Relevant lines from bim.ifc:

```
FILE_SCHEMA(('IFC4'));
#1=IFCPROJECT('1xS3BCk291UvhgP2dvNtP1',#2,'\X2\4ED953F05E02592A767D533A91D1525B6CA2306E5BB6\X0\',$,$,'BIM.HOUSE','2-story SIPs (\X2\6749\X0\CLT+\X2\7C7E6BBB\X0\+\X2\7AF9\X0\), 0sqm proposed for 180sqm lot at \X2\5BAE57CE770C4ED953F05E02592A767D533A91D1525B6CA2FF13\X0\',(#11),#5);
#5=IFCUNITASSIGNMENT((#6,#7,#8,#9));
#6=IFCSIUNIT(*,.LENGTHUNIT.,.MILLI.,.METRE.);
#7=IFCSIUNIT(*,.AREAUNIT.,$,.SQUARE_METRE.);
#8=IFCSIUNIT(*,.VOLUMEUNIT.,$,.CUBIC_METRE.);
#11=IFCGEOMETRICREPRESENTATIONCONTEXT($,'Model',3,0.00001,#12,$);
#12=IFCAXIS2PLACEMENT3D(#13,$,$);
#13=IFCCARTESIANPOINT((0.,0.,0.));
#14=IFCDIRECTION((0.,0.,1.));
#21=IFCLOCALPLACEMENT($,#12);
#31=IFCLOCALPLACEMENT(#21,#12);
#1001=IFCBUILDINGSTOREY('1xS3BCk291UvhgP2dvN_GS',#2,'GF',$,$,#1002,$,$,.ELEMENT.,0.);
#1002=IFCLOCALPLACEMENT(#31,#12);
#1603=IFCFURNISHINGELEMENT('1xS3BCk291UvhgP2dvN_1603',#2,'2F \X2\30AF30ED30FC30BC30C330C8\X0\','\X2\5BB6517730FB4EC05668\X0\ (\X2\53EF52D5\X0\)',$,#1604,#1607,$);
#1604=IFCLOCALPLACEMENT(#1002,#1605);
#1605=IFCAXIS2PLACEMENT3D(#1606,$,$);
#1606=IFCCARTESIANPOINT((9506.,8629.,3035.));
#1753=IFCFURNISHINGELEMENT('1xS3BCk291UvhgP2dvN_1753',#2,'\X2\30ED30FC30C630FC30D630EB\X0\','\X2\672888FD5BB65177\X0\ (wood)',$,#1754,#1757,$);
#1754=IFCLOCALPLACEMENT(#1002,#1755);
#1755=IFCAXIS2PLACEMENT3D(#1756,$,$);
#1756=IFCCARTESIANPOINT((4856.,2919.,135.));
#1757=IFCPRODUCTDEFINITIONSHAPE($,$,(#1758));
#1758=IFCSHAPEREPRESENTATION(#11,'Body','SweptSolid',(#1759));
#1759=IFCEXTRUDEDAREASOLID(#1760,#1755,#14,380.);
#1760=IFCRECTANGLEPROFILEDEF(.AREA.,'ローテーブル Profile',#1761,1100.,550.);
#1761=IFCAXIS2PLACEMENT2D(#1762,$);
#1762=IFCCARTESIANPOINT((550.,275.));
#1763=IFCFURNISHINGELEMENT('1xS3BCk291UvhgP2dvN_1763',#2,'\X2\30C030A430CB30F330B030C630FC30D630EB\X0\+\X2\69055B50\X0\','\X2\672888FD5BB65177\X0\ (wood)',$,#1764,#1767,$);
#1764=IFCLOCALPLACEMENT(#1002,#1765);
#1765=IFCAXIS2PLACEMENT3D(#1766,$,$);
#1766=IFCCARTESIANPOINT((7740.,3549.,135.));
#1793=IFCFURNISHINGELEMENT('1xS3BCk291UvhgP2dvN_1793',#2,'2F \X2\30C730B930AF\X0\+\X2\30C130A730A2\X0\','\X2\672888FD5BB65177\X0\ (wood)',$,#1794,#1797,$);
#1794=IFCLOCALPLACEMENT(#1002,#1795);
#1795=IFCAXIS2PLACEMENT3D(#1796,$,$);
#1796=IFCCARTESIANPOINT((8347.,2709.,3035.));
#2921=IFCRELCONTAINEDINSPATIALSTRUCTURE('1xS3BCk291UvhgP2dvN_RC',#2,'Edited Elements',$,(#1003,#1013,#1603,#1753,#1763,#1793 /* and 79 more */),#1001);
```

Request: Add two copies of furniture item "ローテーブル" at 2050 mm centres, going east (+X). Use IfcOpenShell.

```python
import numpy as np
import ifcopenshell
import ifcopenshell.api.geometry
import ifcopenshell.api.root
import ifcopenshell.util.element
import ifcopenshell.util.placement
import ifcopenshell.util.unit

model = ifcopenshell.open("bim.ifc")
unit_scale = ifcopenshell.util.unit.calculate_unit_scale(model)


def reuse_history(source, copy):
    """copy_class also copies each property set's owner history, people and application; keep the originals."""
    for rel in copy.IsDefinedBy:
        if rel.is_a("IfcRelDefinesByProperties") and (history := rel.RelatingPropertyDefinition.OwnerHistory):
            rel.RelatingPropertyDefinition.OwnerHistory = source.OwnerHistory
            ifcopenshell.util.element.remove_deep2(model, history)


source = model.by_id(1753)
base = ifcopenshell.util.placement.get_local_placement(source.ObjectPlacement)
step = np.array([1.0, 0.0, 0.0]) * 2.05 / unit_scale

for i in range(1, 3):
    copy = ifcopenshell.api.root.copy_class(model, product=source)
    copy.Representation = ifcopenshell.util.element.copy_deep(
        model, source.Representation, exclude=["IfcGeometricRepresentationContext", "IfcRepresentationMap"]
    )
    reuse_history(source, copy)
    matrix = base.copy()
    matrix[:3, 3] += i * step
    print("added at", matrix[:3, 3].round(3) + 0.0)
    ifcopenshell.api.geometry.edit_object_placement(model, product=copy, matrix=matrix, is_si=False)

model.write("bim_rev.ifc")
```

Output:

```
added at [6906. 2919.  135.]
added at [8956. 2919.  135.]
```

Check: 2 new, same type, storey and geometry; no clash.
